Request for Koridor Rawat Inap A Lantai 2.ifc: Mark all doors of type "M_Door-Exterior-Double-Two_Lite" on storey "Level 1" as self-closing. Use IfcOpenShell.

First a look at what the model holds.

```python
import ifcopenshell
import ifcopenshell.util.element

model = ifcopenshell.open("Koridor Rawat Inap A Lantai 2.ifc")
print(model.schema)
storey = next(s for s in model.by_type("IfcBuildingStorey") if s.Name == "Level 1")
doors = [e for e in ifcopenshell.util.element.get_decomposition(storey) if e.is_a("IfcDoor")]
seen = {}
for e in doors:
    element_type = ifcopenshell.util.element.get_type(e)
    key = (element_type.Name if element_type != e and element_type else None, ifcopenshell.util.element.get_pset(e, "Pset_DoorCommon", "SelfClosing"))
    seen[key] = seen.get(key, 0) + 1
for (name, value), count in sorted(seen.items(), key=str):
    print(count, "x", name, "|", value)
```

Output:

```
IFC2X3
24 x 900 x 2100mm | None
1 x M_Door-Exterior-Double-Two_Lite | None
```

```python
import ifcopenshell
import ifcopenshell.api.pset
import ifcopenshell.util.element

model = ifcopenshell.open("Koridor Rawat Inap A Lantai 2.ifc")

storey = next(s for s in model.by_type("IfcBuildingStorey") if s.Name == "Level 1")
doors = [e for e in ifcopenshell.util.element.get_decomposition(storey) if e.is_a("IfcDoor")]

count = 0
for e in doors:
    element_type = ifcopenshell.util.element.get_type(e)
    if element_type in (None, e) or element_type.Name != "M_Door-Exterior-Double-Two_Lite":
        continue
    # add_pset returns the element's existing set when there is one.
    pset = ifcopenshell.api.pset.add_pset(model, product=e, name="Pset_DoorCommon")
    ifcopenshell.api.pset.edit_pset(model, pset=pset, properties={"SelfClosing": True})
    count += 1

print(count, "doors updated")

model.write("Koridor Rawat Inap A Lantai 2_updated.ifc")
```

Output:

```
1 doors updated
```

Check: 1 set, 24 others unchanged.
